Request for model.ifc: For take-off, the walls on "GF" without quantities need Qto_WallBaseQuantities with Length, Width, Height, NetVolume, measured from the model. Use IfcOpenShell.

First a look at what the model holds.

```python
import ifcopenshell
import ifcopenshell.util.element
import ifcopenshell.util.unit

model = ifcopenshell.open("model.ifc")
print(model.schema)
for unit_type in ("LENGTHUNIT", "AREAUNIT", "VOLUMEUNIT"):
    print(unit_type, ifcopenshell.util.unit.calculate_unit_scale(model, unit_type))
storey = next(s for s in model.by_type("IfcBuildingStorey") if s.Name == "GF")
walls = [e for e in ifcopenshell.util.element.get_decomposition(storey) if e.is_a("IfcWall")]
for e in sorted(walls, key=lambda e: e.id()):
    print(e.id(), e.is_a(), e.Name, list(ifcopenshell.util.element.get_psets(e, qtos_only=True)), sep=" | ")
```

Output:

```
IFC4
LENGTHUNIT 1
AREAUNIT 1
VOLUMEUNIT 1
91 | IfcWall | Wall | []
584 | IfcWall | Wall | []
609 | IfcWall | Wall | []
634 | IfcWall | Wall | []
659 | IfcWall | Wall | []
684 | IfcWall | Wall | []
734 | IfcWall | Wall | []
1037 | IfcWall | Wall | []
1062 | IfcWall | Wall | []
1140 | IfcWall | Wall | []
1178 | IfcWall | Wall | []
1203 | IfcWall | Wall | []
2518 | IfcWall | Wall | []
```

```python
import ifcopenshell
import ifcopenshell.api.pset
import ifcopenshell.geom
import ifcopenshell.util.element
import ifcopenshell.util.shape
import ifcopenshell.util.unit

model = ifcopenshell.open("model.ifc")
unit_scale = ifcopenshell.util.unit.calculate_unit_scale(model)
volume_scale = ifcopenshell.util.unit.calculate_unit_scale(model, "VOLUMEUNIT")
settings = ifcopenshell.geom.settings()

storey = next(s for s in model.by_type("IfcBuildingStorey") if s.Name == "GF")
walls = [e for e in ifcopenshell.util.element.get_decomposition(storey) if e.is_a("IfcWall")]

for e in sorted(walls, key=lambda e: e.id()):
    if ifcopenshell.util.element.get_psets(e, qtos_only=True, should_inherit=False):
        continue
    # Geometry comes back in metres, in the element's own axes.
    shape = ifcopenshell.geom.create_shape(settings, e)
    values = {
        "Length": ifcopenshell.util.shape.get_x(shape.geometry) / unit_scale,
        "Width": ifcopenshell.util.shape.get_y(shape.geometry) / unit_scale,
        "Height": ifcopenshell.util.shape.get_z(shape.geometry) / unit_scale,
        "NetVolume": ifcopenshell.util.shape.get_volume(shape.geometry) / volume_scale,
    }
    qto = ifcopenshell.api.pset.add_qto(model, product=e, name="Qto_WallBaseQuantities")
    ifcopenshell.api.pset.edit_qto(model, qto=qto, properties=values)
    print(e.id(), {k: round(v, 3) for k, v in values.items()})

model.write("model_rev.ifc")
```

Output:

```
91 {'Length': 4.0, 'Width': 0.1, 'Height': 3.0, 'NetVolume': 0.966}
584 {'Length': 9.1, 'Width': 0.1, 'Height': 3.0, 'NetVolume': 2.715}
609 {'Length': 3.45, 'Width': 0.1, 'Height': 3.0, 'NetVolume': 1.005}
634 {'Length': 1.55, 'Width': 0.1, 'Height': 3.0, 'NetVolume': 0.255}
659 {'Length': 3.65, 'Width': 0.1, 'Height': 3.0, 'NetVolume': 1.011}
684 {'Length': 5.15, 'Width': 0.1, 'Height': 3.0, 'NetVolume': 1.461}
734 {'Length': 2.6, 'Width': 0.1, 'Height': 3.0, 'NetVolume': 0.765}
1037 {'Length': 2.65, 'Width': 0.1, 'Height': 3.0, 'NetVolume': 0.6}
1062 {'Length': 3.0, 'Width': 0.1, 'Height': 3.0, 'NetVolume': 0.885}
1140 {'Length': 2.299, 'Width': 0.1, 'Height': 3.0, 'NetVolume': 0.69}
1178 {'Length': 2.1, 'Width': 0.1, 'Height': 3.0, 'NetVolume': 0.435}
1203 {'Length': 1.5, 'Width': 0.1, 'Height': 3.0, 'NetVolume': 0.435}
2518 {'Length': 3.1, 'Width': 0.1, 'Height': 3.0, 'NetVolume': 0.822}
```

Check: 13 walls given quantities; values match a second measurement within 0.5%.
